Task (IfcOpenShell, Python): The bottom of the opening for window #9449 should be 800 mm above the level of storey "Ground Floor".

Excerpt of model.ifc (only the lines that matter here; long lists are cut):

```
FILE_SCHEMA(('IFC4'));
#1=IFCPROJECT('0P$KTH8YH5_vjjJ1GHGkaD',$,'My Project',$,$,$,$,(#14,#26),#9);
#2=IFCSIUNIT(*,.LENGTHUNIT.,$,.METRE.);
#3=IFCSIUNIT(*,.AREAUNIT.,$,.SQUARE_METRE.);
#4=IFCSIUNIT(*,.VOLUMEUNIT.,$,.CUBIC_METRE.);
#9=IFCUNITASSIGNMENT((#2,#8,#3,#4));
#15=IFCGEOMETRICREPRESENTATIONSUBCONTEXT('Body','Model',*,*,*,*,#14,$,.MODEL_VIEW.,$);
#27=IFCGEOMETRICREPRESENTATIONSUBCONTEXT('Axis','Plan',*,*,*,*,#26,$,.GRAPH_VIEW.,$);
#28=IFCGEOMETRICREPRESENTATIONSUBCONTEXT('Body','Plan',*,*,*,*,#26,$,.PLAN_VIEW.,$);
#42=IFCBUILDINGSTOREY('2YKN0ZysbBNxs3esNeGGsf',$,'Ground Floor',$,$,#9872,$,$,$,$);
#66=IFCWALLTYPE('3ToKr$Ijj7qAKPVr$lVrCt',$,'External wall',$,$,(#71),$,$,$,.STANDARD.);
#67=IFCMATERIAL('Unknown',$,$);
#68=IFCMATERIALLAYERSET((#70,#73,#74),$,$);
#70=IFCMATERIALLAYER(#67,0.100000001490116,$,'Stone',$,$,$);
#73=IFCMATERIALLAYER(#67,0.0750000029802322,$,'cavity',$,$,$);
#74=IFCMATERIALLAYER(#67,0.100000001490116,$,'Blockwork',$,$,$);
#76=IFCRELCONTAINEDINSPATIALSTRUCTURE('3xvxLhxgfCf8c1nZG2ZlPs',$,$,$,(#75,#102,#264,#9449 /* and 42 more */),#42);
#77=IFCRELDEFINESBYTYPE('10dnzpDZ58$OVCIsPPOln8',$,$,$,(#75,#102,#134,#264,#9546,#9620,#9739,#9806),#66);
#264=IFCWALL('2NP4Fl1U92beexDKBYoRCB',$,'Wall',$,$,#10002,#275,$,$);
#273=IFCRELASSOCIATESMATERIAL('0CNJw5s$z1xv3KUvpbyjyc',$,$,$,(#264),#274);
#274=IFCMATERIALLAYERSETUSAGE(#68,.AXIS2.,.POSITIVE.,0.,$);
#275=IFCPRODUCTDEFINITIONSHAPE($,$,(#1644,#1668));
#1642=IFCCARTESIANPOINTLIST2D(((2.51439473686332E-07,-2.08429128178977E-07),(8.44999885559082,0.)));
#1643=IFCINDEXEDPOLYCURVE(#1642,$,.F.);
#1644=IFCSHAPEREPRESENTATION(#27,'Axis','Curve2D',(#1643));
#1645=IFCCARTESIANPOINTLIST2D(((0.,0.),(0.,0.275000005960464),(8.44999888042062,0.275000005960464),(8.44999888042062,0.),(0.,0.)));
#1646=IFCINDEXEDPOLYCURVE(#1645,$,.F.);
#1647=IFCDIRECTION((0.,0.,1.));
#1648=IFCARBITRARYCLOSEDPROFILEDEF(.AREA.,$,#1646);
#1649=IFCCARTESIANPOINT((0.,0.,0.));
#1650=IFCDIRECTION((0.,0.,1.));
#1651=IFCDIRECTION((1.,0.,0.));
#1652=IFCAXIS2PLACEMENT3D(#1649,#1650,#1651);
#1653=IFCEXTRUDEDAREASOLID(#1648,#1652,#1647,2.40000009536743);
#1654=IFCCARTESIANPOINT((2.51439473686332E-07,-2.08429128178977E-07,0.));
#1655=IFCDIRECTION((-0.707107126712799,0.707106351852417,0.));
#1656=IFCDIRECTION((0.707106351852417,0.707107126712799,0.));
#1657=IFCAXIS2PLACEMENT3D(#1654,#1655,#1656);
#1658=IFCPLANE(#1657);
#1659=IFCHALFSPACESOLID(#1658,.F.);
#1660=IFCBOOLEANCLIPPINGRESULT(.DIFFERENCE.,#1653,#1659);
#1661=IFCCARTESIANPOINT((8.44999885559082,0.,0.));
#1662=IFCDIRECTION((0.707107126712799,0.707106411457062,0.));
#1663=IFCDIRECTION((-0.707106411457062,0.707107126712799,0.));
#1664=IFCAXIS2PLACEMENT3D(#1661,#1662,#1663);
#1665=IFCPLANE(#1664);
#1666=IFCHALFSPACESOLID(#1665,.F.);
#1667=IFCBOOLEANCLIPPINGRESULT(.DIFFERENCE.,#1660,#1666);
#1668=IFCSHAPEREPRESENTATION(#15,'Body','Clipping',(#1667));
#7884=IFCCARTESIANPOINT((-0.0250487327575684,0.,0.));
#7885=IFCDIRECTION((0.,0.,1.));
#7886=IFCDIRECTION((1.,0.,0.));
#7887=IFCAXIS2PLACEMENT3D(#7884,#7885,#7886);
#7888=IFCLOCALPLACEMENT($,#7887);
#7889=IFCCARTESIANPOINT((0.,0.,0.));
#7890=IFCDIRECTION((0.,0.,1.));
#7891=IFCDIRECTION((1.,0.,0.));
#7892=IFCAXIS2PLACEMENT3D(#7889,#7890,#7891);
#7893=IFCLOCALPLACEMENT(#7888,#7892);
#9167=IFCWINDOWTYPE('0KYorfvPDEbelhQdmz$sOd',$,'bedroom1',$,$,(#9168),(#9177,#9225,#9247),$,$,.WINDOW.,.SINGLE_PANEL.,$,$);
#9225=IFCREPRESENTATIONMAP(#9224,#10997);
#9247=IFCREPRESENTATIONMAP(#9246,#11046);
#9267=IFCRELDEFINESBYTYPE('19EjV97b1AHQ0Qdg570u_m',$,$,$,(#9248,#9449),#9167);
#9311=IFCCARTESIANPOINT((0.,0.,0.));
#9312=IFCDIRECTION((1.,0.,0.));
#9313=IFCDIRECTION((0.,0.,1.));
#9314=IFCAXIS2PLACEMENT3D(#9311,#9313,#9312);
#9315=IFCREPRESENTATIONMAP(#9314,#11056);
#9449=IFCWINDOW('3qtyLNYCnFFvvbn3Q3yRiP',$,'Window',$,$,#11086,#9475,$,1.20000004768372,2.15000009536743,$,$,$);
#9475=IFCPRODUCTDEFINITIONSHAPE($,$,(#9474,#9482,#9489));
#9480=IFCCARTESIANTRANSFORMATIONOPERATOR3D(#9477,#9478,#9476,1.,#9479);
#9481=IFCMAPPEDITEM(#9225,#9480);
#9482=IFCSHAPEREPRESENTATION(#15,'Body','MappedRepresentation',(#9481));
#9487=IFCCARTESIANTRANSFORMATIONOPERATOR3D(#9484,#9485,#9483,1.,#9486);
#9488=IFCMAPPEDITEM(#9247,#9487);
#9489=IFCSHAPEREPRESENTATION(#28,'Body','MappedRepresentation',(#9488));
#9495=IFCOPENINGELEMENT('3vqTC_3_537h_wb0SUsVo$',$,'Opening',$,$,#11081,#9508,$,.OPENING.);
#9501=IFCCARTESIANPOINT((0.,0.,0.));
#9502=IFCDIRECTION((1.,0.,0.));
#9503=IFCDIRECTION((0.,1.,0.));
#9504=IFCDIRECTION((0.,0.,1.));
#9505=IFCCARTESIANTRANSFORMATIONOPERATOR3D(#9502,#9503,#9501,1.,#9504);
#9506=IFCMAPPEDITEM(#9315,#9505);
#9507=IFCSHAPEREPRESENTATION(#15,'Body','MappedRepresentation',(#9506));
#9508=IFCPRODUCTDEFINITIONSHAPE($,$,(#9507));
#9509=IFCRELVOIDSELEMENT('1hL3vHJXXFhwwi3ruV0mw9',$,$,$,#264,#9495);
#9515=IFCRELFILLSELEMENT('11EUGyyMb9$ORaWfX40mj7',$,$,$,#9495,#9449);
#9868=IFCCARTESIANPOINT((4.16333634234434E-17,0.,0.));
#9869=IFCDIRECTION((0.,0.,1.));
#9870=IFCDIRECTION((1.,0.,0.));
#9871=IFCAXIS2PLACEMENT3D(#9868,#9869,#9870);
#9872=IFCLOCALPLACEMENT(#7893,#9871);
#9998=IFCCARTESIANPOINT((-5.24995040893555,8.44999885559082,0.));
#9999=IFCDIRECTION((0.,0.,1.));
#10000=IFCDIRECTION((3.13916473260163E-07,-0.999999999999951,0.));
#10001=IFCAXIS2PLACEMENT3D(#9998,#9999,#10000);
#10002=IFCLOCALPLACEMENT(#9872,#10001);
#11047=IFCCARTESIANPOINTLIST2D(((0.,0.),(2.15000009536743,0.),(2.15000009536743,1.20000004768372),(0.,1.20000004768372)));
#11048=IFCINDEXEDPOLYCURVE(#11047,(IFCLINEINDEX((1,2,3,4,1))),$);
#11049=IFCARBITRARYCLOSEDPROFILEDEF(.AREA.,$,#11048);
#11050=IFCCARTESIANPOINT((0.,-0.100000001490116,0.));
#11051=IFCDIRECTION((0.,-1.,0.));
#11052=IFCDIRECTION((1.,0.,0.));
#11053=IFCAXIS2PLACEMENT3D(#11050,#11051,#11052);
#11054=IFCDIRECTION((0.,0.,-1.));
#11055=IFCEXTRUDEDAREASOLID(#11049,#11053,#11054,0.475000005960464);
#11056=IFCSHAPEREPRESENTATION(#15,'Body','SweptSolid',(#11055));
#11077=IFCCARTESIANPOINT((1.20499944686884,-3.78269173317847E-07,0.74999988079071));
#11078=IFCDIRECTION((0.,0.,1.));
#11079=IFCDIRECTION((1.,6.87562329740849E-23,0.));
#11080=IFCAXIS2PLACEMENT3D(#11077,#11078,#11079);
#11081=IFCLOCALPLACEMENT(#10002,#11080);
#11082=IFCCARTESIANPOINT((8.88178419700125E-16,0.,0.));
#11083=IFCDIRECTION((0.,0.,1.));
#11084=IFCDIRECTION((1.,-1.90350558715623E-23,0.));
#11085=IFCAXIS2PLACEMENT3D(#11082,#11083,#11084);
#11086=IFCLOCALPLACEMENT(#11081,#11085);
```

```python
import numpy as np
import ifcopenshell
import ifcopenshell.api.geometry
import ifcopenshell.geom
import ifcopenshell.util.element
import ifcopenshell.util.placement
import ifcopenshell.util.shape
import ifcopenshell.util.unit

model = ifcopenshell.open("model.ifc")
unit_scale = ifcopenshell.util.unit.calculate_unit_scale(model)

window = model.by_guid("3qtyLNYCnFFvvbn3Q3yRiP")
opening = window.FillsVoids[0].RelatingOpeningElement
storey = ifcopenshell.util.element.get_container(window, ifc_class="IfcBuildingStorey")
level = ifcopenshell.util.placement.get_local_placement(storey.ObjectPlacement)[2, 3]

# The opening's origin need not be at the sill, so measure its lowest point.
shape = ifcopenshell.geom.create_shape(ifcopenshell.geom.settings(), opening)
bottom = ifcopenshell.util.shape.get_shape_bottom_elevation(shape, shape.geometry) / unit_scale
dz = level + 0.8 / unit_scale - bottom

shift = np.array([0.0, 0.0, dz])
# The window is placed relative to its opening, so it follows when the opening moves.
matrix = ifcopenshell.util.placement.get_local_placement(opening.ObjectPlacement)
matrix[:3, 3] += shift
ifcopenshell.api.geometry.edit_object_placement(
    model, product=opening, matrix=matrix, is_si=False, should_transform_children=True
)

print(f"moved by {dz * unit_scale:+.3f} m")

model.write("model-out.ifc")
```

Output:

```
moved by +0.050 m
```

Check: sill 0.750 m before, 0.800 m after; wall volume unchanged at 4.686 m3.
